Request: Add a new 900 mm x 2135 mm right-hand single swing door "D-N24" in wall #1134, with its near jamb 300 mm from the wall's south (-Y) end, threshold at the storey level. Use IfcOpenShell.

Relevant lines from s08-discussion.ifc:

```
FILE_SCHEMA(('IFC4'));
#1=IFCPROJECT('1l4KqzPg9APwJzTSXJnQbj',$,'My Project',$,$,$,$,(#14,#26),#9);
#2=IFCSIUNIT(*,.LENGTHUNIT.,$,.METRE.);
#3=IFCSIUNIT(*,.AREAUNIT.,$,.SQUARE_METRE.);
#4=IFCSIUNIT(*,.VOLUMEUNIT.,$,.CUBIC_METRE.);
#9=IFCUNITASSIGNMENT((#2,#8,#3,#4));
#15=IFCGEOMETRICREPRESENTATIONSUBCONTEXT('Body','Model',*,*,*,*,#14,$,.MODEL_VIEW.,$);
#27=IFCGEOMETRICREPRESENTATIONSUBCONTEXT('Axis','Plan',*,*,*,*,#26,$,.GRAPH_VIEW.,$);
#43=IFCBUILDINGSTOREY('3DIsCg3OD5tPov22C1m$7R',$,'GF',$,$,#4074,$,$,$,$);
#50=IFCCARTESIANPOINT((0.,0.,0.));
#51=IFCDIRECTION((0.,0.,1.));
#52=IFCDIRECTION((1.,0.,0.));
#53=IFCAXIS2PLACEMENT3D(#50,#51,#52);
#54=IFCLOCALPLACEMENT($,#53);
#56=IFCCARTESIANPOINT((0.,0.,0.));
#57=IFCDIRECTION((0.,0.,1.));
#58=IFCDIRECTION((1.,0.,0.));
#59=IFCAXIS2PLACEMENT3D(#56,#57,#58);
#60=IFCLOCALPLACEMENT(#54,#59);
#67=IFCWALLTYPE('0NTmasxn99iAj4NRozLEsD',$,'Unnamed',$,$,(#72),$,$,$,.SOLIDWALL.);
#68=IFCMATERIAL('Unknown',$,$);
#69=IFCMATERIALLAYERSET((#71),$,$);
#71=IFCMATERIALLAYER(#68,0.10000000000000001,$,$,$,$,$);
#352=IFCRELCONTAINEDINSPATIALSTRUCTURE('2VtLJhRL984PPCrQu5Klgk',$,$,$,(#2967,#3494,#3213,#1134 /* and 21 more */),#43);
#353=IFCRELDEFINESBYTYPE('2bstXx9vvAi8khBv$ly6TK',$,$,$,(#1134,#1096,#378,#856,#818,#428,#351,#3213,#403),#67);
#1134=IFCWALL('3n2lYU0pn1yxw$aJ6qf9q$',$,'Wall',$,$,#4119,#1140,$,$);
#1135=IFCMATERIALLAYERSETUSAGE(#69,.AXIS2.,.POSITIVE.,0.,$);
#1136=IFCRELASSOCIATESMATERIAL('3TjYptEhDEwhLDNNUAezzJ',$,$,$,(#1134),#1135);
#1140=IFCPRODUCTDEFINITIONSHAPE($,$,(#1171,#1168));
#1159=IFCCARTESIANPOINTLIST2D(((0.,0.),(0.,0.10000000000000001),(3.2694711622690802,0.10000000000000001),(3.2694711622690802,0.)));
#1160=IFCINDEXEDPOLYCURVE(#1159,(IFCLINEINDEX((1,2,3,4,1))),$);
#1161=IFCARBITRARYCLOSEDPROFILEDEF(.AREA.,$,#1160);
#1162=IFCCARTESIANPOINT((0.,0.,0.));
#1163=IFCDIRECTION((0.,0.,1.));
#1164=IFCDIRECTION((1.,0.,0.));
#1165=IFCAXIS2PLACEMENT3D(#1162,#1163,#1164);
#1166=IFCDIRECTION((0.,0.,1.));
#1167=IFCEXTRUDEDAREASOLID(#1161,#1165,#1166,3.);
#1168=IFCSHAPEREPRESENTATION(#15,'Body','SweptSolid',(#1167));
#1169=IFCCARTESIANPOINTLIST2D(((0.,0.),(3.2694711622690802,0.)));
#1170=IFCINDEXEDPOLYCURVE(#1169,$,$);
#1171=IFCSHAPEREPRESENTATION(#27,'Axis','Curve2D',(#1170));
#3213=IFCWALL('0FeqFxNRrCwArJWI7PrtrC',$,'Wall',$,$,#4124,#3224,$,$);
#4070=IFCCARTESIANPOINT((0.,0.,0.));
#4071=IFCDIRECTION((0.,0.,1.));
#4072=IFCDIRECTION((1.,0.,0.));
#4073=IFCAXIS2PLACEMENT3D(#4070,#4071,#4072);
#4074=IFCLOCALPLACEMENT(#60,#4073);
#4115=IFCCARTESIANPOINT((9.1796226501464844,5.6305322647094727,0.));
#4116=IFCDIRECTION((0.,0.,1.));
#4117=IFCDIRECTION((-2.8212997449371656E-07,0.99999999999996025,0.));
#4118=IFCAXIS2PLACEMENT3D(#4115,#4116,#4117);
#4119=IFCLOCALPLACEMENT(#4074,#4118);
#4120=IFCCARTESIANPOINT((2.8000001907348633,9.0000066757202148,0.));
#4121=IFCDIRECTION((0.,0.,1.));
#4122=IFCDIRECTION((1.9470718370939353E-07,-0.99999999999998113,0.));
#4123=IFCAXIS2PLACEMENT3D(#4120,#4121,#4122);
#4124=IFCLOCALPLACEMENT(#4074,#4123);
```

```python
import numpy as np
import ifcopenshell
import ifcopenshell.api.feature
import ifcopenshell.api.geometry
import ifcopenshell.api.root
import ifcopenshell.api.spatial
import ifcopenshell.geom
import ifcopenshell.util.element
import ifcopenshell.util.placement
import ifcopenshell.util.representation
import ifcopenshell.util.shape
import ifcopenshell.util.unit

model = ifcopenshell.open("s08-discussion.ifc")
unit_scale = ifcopenshell.util.unit.calculate_unit_scale(model)
settings = ifcopenshell.geom.settings()


def volume(element):
    """Net volume in cubic metres, openings subtracted."""
    shape = ifcopenshell.geom.create_shape(settings, element)
    return ifcopenshell.util.shape.get_volume(shape.geometry)


wall = model.by_id(1134)
storey = ifcopenshell.util.element.get_container(wall, ifc_class="IfcBuildingStorey")
context = ifcopenshell.util.representation.get_context(model, "Model", "Body", "MODEL_VIEW")
before = volume(wall)

width, height, from_end, sill = 0.9, 2.135, 0.3, 0.0  # metres

# The wall runs along its own X axis, and the end named is its -X end.
wall_shape = ifcopenshell.geom.create_shape(settings, wall)
x, y, z = ifcopenshell.util.shape.get_vertices(wall_shape.geometry).T
start = x.min() + from_end
face, thickness = float(y.min()), float(y.max() - y.min())
wall_matrix = ifcopenshell.util.placement.get_local_placement(wall.ObjectPlacement)
level = ifcopenshell.util.placement.get_local_placement(storey.ObjectPlacement)[2, 3]


def in_wall(x, y):
    """Placement at x, y metres in the wall's axes, at sill height."""
    matrix = wall_matrix.copy()
    matrix[:, 3] = wall_matrix @ np.array([x / unit_scale, y / unit_scale, 0.0, 1.0])
    matrix[2, 3] = level + sill / unit_scale
    return matrix


# Opening: a box that overshoots both wall faces by 50 mm.
opening = ifcopenshell.api.root.create_entity(model, ifc_class="IfcOpeningElement", predefined_type="OPENING")
box = ifcopenshell.api.geometry.add_wall_representation(
    model, context=context, length=width, height=height, thickness=thickness + 0.1
)
ifcopenshell.api.geometry.assign_representation(model, product=opening, representation=box)
ifcopenshell.api.geometry.edit_object_placement(model, product=opening, matrix=in_wall(start, face - 0.05), is_si=False)
ifcopenshell.api.feature.add_feature(model, feature=opening, element=wall)

door = ifcopenshell.api.root.create_entity(model, ifc_class="IfcDoor", name="D-N24", predefined_type="DOOR")
door.OverallWidth, door.OverallHeight = width / unit_scale, height / unit_scale
door.OperationType = "SINGLE_SWING_RIGHT"
body = ifcopenshell.api.geometry.add_door_representation(
    model,
    context=context,
    overall_width=door.OverallWidth,
    overall_height=door.OverallHeight,
    operation_type="SINGLE_SWING_RIGHT",
    lining_properties={"LiningDepth": thickness / unit_scale, "ThresholdDepth": thickness / unit_scale},
)
ifcopenshell.api.geometry.assign_representation(model, product=door, representation=body)
ifcopenshell.api.spatial.assign_container(model, products=[door], relating_structure=storey)
ifcopenshell.api.feature.add_filling(model, opening=opening, element=door)

# The lining spans the wall, so the door starts at the wall face.
ifcopenshell.api.geometry.edit_object_placement(model, product=door, matrix=in_wall(start, face), is_si=False)

after = volume(wall)

print(f"wall volume {before:.3f} -> {after:.3f} m3")

model.write("s08-discussion_v2.ifc")
```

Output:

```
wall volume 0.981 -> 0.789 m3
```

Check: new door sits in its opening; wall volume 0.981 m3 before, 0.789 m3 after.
